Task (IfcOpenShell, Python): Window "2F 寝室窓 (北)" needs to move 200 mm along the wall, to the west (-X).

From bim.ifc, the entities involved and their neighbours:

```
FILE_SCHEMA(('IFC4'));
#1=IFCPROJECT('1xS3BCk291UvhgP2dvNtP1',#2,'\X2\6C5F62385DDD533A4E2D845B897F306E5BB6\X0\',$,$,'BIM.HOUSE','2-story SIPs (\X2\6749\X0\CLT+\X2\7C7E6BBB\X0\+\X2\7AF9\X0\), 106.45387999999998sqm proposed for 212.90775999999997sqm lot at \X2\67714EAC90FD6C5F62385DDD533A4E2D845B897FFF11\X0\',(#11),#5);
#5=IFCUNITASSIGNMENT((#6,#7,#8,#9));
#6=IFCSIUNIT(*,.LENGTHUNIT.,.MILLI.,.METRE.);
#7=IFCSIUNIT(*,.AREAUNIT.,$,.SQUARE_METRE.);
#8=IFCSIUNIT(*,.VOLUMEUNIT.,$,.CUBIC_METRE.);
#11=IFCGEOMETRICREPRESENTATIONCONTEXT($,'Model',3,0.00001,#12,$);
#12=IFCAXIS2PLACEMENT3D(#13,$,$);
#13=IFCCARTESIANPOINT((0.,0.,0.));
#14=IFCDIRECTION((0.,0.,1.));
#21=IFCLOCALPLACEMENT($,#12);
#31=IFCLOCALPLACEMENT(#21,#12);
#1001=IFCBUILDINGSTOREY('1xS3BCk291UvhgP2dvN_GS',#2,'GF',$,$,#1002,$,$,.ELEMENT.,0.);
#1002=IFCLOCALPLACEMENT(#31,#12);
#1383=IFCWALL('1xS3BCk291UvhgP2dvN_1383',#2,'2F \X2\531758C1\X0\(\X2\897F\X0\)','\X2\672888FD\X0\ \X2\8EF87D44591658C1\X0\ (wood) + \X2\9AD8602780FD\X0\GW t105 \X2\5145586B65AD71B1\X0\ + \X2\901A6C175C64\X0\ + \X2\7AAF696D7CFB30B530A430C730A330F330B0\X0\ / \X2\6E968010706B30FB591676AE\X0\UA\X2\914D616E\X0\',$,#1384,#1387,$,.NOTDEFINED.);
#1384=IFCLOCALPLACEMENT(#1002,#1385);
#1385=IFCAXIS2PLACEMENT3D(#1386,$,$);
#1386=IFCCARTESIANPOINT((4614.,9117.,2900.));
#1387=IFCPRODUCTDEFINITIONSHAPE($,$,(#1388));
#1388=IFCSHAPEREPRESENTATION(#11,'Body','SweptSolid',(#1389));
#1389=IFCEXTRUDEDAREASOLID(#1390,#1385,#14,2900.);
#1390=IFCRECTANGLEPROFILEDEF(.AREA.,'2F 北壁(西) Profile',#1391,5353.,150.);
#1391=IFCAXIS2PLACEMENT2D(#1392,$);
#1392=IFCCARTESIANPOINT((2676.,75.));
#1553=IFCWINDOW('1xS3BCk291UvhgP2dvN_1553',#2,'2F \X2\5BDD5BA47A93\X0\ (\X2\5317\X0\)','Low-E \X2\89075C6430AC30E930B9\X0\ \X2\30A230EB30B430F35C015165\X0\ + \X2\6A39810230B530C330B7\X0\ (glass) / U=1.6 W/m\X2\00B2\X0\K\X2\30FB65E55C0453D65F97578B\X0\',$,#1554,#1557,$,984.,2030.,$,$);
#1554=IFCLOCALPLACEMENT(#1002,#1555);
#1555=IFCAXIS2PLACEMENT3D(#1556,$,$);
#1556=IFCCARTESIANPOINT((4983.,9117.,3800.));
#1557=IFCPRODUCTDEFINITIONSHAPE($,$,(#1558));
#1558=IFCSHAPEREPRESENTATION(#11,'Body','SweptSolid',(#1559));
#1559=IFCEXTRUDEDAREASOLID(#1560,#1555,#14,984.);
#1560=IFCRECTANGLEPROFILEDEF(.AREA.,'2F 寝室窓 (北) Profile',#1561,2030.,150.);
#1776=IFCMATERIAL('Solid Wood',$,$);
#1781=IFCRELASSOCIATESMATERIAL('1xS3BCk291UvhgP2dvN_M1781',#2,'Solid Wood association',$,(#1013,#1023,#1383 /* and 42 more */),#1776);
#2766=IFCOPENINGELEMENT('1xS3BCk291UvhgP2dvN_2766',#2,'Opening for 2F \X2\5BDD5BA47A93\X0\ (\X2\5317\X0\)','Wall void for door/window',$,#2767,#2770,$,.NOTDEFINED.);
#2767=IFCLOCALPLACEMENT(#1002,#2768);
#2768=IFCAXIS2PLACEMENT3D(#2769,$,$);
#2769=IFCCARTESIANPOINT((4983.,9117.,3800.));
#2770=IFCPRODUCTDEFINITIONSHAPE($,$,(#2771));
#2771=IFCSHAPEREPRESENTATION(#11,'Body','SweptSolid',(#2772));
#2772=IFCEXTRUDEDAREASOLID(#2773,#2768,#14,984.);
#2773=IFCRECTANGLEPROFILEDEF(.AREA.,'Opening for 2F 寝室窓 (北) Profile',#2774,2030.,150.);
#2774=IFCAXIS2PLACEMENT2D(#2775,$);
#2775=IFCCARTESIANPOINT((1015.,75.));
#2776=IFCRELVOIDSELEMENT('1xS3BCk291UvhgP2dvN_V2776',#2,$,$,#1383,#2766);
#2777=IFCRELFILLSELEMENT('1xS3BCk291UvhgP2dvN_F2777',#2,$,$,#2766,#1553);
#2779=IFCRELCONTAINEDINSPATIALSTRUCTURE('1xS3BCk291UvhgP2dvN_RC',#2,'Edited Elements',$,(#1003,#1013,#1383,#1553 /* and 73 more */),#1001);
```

```python
import ifcopenshell
import ifcopenshell.api.geometry
import ifcopenshell.util.placement

model = ifcopenshell.open("bim.ifc")

window = model.by_guid("1xS3BCk291UvhgP2dvN_1553")
opening = window.FillsVoids[0].RelatingOpeningElement
wall = opening.VoidsElements[0].RelatingBuildingElement

wall_matrix = ifcopenshell.util.placement.get_local_placement(wall.ObjectPlacement)
shift = wall_matrix[:3, 0] * -200.0
before = ifcopenshell.util.placement.get_local_placement(window.ObjectPlacement)[:3, 3].copy()

# The window is not placed relative to its opening, so move both.
for product in (opening, window):
    matrix = ifcopenshell.util.placement.get_local_placement(product.ObjectPlacement)
    matrix[:3, 3] += shift
    ifcopenshell.api.geometry.edit_object_placement(model, product=product, matrix=matrix, is_si=False)

after = ifcopenshell.util.placement.get_local_placement(window.ObjectPlacement)[:3, 3]
print("window moved by", (after - before).round(3) + 0.0)

model.write("bim_edited.ifc")
```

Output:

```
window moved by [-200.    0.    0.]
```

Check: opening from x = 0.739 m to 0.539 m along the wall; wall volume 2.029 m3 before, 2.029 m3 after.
